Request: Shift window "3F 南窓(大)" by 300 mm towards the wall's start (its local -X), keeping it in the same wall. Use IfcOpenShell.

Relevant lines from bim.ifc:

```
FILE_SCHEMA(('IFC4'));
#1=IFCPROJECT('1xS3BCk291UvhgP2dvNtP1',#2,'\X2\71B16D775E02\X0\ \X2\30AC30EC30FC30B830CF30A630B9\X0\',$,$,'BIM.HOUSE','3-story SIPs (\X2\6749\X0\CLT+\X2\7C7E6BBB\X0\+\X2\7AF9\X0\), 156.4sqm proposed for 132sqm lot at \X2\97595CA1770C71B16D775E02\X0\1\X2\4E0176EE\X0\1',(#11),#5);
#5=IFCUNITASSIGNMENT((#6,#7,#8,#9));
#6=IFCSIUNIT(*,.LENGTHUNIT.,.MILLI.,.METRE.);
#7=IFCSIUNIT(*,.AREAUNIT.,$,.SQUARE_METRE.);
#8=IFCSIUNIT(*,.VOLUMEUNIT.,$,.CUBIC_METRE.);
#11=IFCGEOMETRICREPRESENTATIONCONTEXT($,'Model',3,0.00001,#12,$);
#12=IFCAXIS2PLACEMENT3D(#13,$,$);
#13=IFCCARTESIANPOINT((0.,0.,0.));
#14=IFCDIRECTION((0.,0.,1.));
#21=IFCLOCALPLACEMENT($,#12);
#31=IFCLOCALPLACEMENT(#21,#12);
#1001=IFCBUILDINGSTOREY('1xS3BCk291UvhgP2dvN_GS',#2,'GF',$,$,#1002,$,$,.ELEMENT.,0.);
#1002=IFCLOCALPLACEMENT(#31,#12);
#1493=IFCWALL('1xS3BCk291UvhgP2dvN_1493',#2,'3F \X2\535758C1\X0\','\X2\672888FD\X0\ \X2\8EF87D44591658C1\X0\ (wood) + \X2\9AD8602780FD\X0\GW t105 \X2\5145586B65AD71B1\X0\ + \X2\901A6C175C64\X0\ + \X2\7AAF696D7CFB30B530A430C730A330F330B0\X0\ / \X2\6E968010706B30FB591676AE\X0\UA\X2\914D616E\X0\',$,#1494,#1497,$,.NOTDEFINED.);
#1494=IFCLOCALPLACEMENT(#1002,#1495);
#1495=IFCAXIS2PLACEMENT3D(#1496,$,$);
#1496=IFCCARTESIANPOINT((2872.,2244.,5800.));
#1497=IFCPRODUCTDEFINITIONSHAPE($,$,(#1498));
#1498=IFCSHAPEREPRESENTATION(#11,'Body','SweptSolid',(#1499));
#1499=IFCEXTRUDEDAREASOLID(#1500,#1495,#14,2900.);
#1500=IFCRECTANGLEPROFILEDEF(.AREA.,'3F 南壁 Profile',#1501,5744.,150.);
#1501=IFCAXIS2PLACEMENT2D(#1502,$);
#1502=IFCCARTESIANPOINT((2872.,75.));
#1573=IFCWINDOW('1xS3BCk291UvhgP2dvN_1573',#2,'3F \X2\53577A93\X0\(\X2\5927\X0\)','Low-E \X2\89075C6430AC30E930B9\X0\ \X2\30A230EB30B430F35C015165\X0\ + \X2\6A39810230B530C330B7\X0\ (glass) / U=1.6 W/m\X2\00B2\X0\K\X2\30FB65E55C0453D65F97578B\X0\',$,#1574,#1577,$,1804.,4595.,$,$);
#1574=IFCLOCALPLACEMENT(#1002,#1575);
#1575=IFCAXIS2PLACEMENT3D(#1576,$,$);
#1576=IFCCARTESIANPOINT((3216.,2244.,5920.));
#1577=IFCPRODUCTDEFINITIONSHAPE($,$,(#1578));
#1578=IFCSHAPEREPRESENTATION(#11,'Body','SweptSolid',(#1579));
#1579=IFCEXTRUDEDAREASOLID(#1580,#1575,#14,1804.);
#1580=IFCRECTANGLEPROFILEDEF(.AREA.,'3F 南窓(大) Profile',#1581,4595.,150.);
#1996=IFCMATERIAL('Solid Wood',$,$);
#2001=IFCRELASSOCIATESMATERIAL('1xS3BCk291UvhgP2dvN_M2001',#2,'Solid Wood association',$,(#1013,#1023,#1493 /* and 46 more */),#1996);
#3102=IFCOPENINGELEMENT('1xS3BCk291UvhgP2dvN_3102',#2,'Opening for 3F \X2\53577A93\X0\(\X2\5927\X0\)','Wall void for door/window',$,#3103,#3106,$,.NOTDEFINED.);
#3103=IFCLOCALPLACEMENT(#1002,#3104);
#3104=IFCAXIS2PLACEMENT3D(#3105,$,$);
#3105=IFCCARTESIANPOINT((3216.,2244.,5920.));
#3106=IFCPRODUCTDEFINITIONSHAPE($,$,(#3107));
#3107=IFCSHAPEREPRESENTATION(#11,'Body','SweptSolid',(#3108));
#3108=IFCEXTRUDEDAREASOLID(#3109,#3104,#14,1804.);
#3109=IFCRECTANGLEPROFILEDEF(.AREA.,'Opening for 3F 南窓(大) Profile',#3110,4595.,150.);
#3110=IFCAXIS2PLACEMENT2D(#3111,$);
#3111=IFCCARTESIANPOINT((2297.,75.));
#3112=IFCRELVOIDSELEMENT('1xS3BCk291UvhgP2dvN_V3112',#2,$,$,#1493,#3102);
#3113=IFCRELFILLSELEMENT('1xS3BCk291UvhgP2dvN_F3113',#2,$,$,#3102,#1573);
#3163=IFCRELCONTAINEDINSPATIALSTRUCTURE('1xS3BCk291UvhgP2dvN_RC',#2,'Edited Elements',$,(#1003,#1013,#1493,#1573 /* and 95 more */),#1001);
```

```python
import ifcopenshell
import ifcopenshell.api.geometry
import ifcopenshell.util.placement
import ifcopenshell.util.unit

model = ifcopenshell.open("bim.ifc")
unit_scale = ifcopenshell.util.unit.calculate_unit_scale(model)

window = model.by_guid("1xS3BCk291UvhgP2dvN_1573")
opening = window.FillsVoids[0].RelatingOpeningElement
wall = opening.VoidsElements[0].RelatingBuildingElement

wall_matrix = ifcopenshell.util.placement.get_local_placement(wall.ObjectPlacement)
shift = wall_matrix[:3, 0] * -0.3 / unit_scale
before = ifcopenshell.util.placement.get_local_placement(window.ObjectPlacement)[:3, 3].copy()

# The window is not placed relative to its opening, so move both.
for product in (opening, window):
    matrix = ifcopenshell.util.placement.get_local_placement(product.ObjectPlacement)
    matrix[:3, 3] += shift
    ifcopenshell.api.geometry.edit_object_placement(model, product=product, matrix=matrix, is_si=False)

after = ifcopenshell.util.placement.get_local_placement(window.ObjectPlacement)[:3, 3]
print("window moved by", (after - before).round(3) + 0.0)

model.write("bim_updated.ifc")
```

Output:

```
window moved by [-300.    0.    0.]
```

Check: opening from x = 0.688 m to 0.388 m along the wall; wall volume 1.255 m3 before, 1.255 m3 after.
